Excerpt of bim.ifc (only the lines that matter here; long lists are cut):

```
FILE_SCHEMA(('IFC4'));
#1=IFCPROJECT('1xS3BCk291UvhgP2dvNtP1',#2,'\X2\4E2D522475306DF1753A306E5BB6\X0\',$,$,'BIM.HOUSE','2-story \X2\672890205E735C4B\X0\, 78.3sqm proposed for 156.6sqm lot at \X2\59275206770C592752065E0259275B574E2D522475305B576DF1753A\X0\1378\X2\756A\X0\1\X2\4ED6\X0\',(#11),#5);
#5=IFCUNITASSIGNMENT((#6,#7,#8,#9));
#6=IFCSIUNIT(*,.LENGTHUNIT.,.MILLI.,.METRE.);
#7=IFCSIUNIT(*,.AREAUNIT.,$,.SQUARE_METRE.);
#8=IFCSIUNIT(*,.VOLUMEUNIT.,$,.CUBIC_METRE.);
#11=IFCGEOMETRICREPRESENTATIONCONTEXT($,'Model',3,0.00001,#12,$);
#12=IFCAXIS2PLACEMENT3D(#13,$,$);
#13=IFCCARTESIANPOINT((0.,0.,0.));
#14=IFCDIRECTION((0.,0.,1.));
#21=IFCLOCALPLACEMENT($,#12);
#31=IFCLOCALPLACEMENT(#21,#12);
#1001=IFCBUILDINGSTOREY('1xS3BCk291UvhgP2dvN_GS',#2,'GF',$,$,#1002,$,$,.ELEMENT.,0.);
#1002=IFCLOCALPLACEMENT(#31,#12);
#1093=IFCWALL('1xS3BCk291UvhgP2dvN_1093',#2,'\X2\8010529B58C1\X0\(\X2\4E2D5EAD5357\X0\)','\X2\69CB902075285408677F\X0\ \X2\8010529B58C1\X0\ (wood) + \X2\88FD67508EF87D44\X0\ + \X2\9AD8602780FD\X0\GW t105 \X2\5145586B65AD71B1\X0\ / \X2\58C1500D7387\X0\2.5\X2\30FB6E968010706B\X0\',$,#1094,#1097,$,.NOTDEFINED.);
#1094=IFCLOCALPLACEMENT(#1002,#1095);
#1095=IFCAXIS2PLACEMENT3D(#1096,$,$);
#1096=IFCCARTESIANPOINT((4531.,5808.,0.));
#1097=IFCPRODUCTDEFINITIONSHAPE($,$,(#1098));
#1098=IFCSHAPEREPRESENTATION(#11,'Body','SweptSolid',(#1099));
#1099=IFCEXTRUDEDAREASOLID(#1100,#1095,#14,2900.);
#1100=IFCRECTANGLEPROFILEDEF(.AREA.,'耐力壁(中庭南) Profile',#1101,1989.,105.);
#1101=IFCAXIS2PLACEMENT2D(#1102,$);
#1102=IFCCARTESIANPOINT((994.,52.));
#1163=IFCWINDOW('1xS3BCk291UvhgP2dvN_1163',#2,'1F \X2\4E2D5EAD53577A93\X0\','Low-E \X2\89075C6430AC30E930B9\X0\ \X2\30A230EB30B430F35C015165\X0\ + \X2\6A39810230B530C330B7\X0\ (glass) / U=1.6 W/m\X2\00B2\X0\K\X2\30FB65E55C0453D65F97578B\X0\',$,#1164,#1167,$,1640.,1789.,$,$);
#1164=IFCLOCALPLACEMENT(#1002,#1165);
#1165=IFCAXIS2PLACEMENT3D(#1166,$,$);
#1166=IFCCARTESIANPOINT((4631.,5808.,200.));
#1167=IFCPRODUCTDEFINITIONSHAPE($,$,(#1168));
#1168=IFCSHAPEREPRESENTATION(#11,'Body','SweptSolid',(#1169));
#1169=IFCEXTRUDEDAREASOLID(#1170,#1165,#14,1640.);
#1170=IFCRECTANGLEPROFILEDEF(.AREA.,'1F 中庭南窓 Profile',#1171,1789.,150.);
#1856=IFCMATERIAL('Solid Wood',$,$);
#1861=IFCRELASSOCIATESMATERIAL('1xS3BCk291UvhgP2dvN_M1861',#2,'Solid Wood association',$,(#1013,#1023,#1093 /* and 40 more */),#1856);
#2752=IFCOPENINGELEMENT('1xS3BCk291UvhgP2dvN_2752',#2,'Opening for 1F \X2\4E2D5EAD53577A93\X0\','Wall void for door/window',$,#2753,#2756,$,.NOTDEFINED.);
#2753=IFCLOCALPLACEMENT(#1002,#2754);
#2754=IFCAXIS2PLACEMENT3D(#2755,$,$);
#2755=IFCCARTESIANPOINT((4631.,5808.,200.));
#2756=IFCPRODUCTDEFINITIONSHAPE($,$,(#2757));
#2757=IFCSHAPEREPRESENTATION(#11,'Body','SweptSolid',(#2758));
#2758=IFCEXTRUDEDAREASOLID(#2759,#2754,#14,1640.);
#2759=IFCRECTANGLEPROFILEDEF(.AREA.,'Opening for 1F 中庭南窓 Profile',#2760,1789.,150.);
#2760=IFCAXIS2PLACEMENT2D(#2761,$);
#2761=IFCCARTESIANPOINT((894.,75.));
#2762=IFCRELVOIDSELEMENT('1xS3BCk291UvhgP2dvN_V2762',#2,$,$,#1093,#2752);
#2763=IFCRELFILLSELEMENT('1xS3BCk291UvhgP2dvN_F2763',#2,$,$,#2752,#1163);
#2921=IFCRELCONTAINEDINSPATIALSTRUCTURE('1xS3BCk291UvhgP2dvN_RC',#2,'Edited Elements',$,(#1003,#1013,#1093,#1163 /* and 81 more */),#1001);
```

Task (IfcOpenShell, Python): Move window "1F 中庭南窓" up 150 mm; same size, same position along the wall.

```python
import numpy as np
import ifcopenshell
import ifcopenshell.api.geometry
import ifcopenshell.util.placement
import ifcopenshell.util.unit

model = ifcopenshell.open("bim.ifc")
unit_scale = ifcopenshell.util.unit.calculate_unit_scale(model)

window = model.by_guid("1xS3BCk291UvhgP2dvN_1163")
opening = window.FillsVoids[0].RelatingOpeningElement
dz = 150.0

shift = np.array([0.0, 0.0, dz])
# The window is not placed relative to its opening, so move both.
for product in (opening, window):
    matrix = ifcopenshell.util.placement.get_local_placement(product.ObjectPlacement)
    matrix[:3, 3] += shift
    ifcopenshell.api.geometry.edit_object_placement(model, product=product, matrix=matrix, is_si=False)

print(f"moved by {dz * unit_scale:+.3f} m")

model.write("bim_edited.ifc")
```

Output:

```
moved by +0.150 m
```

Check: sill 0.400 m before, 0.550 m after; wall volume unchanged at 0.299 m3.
